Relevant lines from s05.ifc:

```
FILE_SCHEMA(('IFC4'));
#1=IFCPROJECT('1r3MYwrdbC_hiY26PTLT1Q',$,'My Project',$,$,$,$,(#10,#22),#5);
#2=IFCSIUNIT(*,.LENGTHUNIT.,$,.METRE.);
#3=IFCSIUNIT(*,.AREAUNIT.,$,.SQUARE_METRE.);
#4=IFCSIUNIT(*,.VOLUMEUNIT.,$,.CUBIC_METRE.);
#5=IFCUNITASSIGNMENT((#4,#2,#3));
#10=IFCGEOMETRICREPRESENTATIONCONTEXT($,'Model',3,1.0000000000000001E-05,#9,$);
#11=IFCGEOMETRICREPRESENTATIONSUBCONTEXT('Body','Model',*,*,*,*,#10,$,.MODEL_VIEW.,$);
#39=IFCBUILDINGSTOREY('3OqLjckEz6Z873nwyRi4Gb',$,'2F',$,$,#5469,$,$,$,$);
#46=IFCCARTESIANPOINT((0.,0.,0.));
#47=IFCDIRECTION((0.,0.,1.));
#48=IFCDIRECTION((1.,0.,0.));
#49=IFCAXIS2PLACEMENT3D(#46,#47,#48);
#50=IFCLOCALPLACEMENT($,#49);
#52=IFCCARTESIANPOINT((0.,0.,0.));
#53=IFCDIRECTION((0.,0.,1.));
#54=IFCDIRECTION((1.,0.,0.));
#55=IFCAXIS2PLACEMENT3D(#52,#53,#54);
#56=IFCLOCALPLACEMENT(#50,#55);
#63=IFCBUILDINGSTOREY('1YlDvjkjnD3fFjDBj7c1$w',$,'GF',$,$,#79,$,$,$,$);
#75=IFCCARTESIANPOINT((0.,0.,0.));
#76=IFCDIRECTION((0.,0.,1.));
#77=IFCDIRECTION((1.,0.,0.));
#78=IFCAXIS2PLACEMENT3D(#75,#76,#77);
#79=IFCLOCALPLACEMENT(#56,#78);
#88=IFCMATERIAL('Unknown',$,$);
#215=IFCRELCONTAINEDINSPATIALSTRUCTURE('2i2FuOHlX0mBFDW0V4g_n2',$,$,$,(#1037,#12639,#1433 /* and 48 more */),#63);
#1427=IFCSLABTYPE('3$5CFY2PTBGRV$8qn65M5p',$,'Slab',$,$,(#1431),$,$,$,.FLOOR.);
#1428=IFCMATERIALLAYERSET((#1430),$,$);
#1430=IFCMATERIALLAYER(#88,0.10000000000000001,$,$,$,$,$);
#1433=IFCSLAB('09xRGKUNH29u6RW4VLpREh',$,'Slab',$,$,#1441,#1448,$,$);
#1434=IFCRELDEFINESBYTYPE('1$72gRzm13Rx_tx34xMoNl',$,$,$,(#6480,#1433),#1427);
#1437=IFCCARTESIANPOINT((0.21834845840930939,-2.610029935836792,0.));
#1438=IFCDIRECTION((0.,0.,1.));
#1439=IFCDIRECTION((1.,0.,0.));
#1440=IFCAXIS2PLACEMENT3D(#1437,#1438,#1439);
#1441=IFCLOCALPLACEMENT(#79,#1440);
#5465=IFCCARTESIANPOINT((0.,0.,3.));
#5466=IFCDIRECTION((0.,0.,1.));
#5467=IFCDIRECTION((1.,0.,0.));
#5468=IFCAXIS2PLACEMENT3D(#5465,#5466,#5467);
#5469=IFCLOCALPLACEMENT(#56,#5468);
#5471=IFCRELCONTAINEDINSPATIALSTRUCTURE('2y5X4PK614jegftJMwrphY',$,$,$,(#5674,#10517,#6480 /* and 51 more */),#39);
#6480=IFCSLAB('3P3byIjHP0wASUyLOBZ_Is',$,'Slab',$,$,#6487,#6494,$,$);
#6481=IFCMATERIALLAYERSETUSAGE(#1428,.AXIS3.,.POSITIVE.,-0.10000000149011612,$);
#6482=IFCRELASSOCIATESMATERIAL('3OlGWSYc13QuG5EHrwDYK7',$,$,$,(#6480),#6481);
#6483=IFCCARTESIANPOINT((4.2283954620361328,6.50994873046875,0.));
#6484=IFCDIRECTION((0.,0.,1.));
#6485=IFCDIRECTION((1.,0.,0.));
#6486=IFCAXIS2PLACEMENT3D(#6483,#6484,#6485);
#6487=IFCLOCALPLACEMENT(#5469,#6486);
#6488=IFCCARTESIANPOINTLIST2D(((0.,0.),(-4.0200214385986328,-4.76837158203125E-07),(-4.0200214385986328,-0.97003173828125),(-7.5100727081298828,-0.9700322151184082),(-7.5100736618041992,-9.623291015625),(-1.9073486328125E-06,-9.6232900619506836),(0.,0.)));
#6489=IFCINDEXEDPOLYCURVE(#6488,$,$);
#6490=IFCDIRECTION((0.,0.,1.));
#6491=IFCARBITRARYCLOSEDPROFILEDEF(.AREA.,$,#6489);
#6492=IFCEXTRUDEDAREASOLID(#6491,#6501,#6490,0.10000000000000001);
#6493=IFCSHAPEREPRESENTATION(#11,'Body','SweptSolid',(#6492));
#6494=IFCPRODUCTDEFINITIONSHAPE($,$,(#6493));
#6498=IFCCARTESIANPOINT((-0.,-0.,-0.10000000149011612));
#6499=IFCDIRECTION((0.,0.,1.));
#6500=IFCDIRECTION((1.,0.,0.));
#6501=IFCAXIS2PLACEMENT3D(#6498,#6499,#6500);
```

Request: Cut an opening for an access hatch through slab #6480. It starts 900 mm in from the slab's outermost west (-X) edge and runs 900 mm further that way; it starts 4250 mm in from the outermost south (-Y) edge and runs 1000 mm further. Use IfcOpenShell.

```python
import numpy as np
import ifcopenshell
import ifcopenshell.api.feature
import ifcopenshell.api.geometry
import ifcopenshell.api.root
import ifcopenshell.geom
import ifcopenshell.util.placement
import ifcopenshell.util.representation
import ifcopenshell.util.shape
import ifcopenshell.util.unit

model = ifcopenshell.open("s05.ifc")
unit_scale = ifcopenshell.util.unit.calculate_unit_scale(model)
settings = ifcopenshell.geom.settings()


def volume(element):
    """Net volume in cubic metres, openings subtracted."""
    shape = ifcopenshell.geom.create_shape(settings, element)
    return ifcopenshell.util.shape.get_volume(shape.geometry)


slab = model.by_guid("3P3byIjHP0wASUyLOBZ_Is")
before = volume(slab)

# Extent in the slab's own axes, in metres. The edges named are its -X and -Y sides.
slab_shape = ifcopenshell.geom.create_shape(settings, slab)
vertices = ifcopenshell.util.shape.get_vertices(slab_shape.geometry)
x_min, y_min, bottom = vertices.min(axis=0)
top = vertices[:, 2].max()

opening = ifcopenshell.api.root.create_entity(model, ifc_class="IfcOpeningElement", name="Access hatch opening", predefined_type="OPENING")
context = ifcopenshell.util.representation.get_context(model, "Model", "Body", "MODEL_VIEW")
width, depth = 0.9, 1
outline = [(0.0, 0.0), (width, 0.0), (width, depth), (0.0, depth), (0.0, 0.0)]
# Overshoot both faces by 50 mm so the cut is clean.
shape = ifcopenshell.api.geometry.add_slab_representation(
    model, context=context, depth=top - bottom + 0.1, polyline=outline
)
ifcopenshell.api.geometry.assign_representation(model, product=opening, representation=shape)

matrix = ifcopenshell.util.placement.get_local_placement(slab.ObjectPlacement)
matrix[:, 3] = matrix @ np.append(np.array([x_min + 0.9, y_min + 4.25, bottom - 0.05]) / unit_scale, 1.0)
ifcopenshell.api.geometry.edit_object_placement(model, product=opening, matrix=matrix, is_si=False)
ifcopenshell.api.feature.add_feature(model, feature=opening, element=slab)

after = volume(slab)

print(f"slab volume {before:.3f} -> {after:.3f} m3")

model.write("s05_v2.ifc")
```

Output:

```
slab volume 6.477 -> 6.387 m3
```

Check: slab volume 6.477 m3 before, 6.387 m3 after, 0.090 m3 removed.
